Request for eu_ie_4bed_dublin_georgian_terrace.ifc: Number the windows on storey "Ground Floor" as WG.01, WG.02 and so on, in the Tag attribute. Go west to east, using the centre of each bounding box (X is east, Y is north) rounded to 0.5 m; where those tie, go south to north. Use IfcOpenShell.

First a look at what the model holds.

```python
import ifcopenshell
import ifcopenshell.util.element
import ifcopenshell.util.placement

model = ifcopenshell.open("eu_ie_4bed_dublin_georgian_terrace.ifc")
print(model.schema)
storey = next(s for s in model.by_type("IfcBuildingStorey") if s.Name == "Ground Floor")
windows = [e for e in ifcopenshell.util.element.get_decomposition(storey) if e.is_a("IfcWindow")]
for e in sorted(windows, key=lambda e: e.id()):
    origin = ifcopenshell.util.placement.get_local_placement(e.ObjectPlacement)[:3, 3]
    print(e.id(), e.Tag, e.Name, origin.round(2) + 0.0, sep=" | ")
```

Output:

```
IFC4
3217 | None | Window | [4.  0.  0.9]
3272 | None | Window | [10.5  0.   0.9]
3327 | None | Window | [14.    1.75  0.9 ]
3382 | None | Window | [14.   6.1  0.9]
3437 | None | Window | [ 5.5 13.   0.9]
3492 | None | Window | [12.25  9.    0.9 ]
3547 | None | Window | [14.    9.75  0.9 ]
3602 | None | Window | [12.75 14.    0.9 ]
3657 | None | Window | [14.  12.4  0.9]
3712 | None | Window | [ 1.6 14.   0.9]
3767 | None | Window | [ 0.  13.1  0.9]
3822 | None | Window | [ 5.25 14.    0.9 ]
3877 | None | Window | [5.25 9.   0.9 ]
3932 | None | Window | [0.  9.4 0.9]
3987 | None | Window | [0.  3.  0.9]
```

```python
import ifcopenshell
import ifcopenshell.geom
import ifcopenshell.util.element
import ifcopenshell.util.shape

model = ifcopenshell.open("eu_ie_4bed_dublin_georgian_terrace.ifc")
settings = ifcopenshell.geom.settings()
settings.set("use-world-coords", True)


def centre(element):
    shape = ifcopenshell.geom.create_shape(settings, element)
    return ifcopenshell.util.shape.get_bbox_centroid(shape.geometry)


storey = next(s for s in model.by_type("IfcBuildingStorey") if s.Name == "Ground Floor")
windows = [e for e in ifcopenshell.util.element.get_decomposition(storey) if e.is_a("IfcWindow")]

# Insertion points can sit at a corner or the storey origin, so sort by the geometry (in metres).
centres = {e: centre(e) for e in windows}
windows.sort(key=lambda e: (round(centres[e][0] / 0.5), centres[e][1]))

for i, e in enumerate(windows, start=1):
    number = f"WG.{i:02d}"
    e.Tag = number
    print(e.id(), number)

model.write("eu_ie_4bed_dublin_georgian_terrace_edited.ifc")
```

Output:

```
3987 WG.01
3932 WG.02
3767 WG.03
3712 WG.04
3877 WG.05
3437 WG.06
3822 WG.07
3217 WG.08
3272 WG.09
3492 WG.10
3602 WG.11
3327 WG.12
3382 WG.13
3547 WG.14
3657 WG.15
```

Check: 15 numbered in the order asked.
